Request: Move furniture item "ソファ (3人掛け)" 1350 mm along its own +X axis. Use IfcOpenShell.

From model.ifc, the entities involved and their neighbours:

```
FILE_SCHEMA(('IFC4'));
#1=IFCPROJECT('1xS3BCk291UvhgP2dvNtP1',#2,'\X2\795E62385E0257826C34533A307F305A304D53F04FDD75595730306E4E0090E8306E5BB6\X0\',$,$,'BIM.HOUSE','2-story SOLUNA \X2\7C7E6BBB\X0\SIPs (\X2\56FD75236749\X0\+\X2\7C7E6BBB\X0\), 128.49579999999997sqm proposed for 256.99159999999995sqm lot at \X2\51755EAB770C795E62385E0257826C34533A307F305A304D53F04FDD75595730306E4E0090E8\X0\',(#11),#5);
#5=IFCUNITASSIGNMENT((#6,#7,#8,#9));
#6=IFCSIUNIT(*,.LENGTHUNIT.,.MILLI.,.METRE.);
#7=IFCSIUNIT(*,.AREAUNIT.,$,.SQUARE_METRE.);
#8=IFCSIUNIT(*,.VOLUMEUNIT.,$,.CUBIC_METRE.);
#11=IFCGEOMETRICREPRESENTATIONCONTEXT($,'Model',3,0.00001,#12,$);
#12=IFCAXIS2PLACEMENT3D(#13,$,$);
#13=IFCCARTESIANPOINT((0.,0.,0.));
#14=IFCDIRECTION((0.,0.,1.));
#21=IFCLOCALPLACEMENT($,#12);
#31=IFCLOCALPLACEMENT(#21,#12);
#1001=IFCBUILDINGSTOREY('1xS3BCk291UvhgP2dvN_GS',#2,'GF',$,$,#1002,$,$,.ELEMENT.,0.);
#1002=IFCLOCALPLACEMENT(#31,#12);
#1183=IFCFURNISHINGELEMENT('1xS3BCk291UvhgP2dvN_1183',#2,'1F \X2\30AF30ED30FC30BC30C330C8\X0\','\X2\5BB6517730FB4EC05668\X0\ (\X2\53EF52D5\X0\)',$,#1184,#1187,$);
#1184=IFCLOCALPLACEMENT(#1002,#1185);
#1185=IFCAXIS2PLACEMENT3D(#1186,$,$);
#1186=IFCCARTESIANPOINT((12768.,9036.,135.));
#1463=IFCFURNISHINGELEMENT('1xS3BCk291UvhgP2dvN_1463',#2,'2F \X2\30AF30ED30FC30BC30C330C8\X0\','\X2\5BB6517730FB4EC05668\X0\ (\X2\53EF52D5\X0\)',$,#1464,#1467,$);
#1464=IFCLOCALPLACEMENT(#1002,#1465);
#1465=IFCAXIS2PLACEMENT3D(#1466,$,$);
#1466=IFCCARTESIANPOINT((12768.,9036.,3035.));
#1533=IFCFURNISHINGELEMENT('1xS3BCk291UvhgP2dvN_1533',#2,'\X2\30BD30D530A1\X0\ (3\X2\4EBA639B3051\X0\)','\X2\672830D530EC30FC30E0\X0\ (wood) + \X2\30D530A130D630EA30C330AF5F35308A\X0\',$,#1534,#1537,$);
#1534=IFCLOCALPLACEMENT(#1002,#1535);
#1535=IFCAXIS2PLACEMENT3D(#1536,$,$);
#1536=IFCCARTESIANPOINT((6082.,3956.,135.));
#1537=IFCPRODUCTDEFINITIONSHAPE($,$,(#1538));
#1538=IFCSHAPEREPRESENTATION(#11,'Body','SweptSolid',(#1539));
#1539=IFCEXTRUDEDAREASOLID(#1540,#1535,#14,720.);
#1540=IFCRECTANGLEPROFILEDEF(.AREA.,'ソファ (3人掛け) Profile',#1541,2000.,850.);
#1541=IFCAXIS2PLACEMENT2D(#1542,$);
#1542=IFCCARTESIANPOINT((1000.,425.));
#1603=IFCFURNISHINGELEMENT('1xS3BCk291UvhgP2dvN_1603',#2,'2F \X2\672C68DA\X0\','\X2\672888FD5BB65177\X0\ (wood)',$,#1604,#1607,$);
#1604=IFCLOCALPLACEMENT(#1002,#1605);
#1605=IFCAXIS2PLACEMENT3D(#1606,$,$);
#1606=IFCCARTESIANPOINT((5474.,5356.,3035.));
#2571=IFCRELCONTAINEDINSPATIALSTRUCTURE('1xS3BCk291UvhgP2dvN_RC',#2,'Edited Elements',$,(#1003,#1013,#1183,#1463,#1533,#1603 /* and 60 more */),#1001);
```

```python
import ifcopenshell
import ifcopenshell.api.geometry
import ifcopenshell.util.placement

model = ifcopenshell.open("model.ifc")

item = model.by_guid("1xS3BCk291UvhgP2dvN_1533")
matrix = ifcopenshell.util.placement.get_local_placement(item.ObjectPlacement)
matrix[:3, 3] += matrix[:3, 0] * 1350.0
ifcopenshell.api.geometry.edit_object_placement(model, product=item, matrix=matrix, is_si=False)

print(ifcopenshell.util.placement.get_local_placement(item.ObjectPlacement).round(3) + 0.0)

model.write("model-out.ifc")
```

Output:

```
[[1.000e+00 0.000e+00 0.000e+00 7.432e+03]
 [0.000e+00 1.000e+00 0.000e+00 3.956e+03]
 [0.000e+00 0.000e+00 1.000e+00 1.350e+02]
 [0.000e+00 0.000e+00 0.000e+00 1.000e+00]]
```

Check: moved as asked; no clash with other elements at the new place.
